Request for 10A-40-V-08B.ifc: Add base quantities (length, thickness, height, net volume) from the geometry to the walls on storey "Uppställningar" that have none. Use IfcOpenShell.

First a look at what the model holds.

```python
import ifcopenshell
import ifcopenshell.util.element
import ifcopenshell.util.unit

model = ifcopenshell.open("10A-40-V-08B.ifc")
print(model.schema)
for unit_type in ("LENGTHUNIT", "AREAUNIT", "VOLUMEUNIT"):
    print(unit_type, ifcopenshell.util.unit.calculate_unit_scale(model, unit_type))
storey = next(s for s in model.by_type("IfcBuildingStorey") if s.Name == "Uppställningar")
walls = [e for e in ifcopenshell.util.element.get_decomposition(storey) if e.is_a("IfcWall")]
for e in sorted(walls, key=lambda e: e.id()):
    print(e.id(), e.is_a(), e.Name, list(ifcopenshell.util.element.get_psets(e, qtos_only=True)), sep=" | ")
```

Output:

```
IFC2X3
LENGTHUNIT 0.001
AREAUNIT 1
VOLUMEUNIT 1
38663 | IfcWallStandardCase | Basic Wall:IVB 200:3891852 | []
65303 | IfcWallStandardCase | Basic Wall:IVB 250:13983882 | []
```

```python
import ifcopenshell
import ifcopenshell.api.pset
import ifcopenshell.geom
import ifcopenshell.util.element
import ifcopenshell.util.shape
import ifcopenshell.util.unit

model = ifcopenshell.open("10A-40-V-08B.ifc")
unit_scale = ifcopenshell.util.unit.calculate_unit_scale(model)
volume_scale = ifcopenshell.util.unit.calculate_unit_scale(model, "VOLUMEUNIT")
settings = ifcopenshell.geom.settings()

storey = next(s for s in model.by_type("IfcBuildingStorey") if s.Name == "Uppställningar")
walls = [e for e in ifcopenshell.util.element.get_decomposition(storey) if e.is_a("IfcWall")]

for e in sorted(walls, key=lambda e: e.id()):
    if ifcopenshell.util.element.get_psets(e, qtos_only=True, should_inherit=False):
        continue
    # Geometry comes back in metres, in the element's own axes.
    shape = ifcopenshell.geom.create_shape(settings, e)
    values = {
        "Length": ifcopenshell.util.shape.get_x(shape.geometry) / unit_scale,
        "Width": ifcopenshell.util.shape.get_y(shape.geometry) / unit_scale,
        "Height": ifcopenshell.util.shape.get_z(shape.geometry) / unit_scale,
        "NetVolume": ifcopenshell.util.shape.get_volume(shape.geometry) / volume_scale,
    }
    qto = ifcopenshell.api.pset.add_qto(model, product=e, name="BaseQuantities")
    ifcopenshell.api.pset.edit_qto(model, qto=qto, properties=values)
    print(e.id(), {k: round(v, 3) for k, v in values.items()})

model.write("10A-40-V-08B-out.ifc")
```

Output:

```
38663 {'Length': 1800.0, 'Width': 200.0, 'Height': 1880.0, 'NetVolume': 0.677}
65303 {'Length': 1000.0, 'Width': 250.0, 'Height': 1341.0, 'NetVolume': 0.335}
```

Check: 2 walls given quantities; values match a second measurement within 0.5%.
